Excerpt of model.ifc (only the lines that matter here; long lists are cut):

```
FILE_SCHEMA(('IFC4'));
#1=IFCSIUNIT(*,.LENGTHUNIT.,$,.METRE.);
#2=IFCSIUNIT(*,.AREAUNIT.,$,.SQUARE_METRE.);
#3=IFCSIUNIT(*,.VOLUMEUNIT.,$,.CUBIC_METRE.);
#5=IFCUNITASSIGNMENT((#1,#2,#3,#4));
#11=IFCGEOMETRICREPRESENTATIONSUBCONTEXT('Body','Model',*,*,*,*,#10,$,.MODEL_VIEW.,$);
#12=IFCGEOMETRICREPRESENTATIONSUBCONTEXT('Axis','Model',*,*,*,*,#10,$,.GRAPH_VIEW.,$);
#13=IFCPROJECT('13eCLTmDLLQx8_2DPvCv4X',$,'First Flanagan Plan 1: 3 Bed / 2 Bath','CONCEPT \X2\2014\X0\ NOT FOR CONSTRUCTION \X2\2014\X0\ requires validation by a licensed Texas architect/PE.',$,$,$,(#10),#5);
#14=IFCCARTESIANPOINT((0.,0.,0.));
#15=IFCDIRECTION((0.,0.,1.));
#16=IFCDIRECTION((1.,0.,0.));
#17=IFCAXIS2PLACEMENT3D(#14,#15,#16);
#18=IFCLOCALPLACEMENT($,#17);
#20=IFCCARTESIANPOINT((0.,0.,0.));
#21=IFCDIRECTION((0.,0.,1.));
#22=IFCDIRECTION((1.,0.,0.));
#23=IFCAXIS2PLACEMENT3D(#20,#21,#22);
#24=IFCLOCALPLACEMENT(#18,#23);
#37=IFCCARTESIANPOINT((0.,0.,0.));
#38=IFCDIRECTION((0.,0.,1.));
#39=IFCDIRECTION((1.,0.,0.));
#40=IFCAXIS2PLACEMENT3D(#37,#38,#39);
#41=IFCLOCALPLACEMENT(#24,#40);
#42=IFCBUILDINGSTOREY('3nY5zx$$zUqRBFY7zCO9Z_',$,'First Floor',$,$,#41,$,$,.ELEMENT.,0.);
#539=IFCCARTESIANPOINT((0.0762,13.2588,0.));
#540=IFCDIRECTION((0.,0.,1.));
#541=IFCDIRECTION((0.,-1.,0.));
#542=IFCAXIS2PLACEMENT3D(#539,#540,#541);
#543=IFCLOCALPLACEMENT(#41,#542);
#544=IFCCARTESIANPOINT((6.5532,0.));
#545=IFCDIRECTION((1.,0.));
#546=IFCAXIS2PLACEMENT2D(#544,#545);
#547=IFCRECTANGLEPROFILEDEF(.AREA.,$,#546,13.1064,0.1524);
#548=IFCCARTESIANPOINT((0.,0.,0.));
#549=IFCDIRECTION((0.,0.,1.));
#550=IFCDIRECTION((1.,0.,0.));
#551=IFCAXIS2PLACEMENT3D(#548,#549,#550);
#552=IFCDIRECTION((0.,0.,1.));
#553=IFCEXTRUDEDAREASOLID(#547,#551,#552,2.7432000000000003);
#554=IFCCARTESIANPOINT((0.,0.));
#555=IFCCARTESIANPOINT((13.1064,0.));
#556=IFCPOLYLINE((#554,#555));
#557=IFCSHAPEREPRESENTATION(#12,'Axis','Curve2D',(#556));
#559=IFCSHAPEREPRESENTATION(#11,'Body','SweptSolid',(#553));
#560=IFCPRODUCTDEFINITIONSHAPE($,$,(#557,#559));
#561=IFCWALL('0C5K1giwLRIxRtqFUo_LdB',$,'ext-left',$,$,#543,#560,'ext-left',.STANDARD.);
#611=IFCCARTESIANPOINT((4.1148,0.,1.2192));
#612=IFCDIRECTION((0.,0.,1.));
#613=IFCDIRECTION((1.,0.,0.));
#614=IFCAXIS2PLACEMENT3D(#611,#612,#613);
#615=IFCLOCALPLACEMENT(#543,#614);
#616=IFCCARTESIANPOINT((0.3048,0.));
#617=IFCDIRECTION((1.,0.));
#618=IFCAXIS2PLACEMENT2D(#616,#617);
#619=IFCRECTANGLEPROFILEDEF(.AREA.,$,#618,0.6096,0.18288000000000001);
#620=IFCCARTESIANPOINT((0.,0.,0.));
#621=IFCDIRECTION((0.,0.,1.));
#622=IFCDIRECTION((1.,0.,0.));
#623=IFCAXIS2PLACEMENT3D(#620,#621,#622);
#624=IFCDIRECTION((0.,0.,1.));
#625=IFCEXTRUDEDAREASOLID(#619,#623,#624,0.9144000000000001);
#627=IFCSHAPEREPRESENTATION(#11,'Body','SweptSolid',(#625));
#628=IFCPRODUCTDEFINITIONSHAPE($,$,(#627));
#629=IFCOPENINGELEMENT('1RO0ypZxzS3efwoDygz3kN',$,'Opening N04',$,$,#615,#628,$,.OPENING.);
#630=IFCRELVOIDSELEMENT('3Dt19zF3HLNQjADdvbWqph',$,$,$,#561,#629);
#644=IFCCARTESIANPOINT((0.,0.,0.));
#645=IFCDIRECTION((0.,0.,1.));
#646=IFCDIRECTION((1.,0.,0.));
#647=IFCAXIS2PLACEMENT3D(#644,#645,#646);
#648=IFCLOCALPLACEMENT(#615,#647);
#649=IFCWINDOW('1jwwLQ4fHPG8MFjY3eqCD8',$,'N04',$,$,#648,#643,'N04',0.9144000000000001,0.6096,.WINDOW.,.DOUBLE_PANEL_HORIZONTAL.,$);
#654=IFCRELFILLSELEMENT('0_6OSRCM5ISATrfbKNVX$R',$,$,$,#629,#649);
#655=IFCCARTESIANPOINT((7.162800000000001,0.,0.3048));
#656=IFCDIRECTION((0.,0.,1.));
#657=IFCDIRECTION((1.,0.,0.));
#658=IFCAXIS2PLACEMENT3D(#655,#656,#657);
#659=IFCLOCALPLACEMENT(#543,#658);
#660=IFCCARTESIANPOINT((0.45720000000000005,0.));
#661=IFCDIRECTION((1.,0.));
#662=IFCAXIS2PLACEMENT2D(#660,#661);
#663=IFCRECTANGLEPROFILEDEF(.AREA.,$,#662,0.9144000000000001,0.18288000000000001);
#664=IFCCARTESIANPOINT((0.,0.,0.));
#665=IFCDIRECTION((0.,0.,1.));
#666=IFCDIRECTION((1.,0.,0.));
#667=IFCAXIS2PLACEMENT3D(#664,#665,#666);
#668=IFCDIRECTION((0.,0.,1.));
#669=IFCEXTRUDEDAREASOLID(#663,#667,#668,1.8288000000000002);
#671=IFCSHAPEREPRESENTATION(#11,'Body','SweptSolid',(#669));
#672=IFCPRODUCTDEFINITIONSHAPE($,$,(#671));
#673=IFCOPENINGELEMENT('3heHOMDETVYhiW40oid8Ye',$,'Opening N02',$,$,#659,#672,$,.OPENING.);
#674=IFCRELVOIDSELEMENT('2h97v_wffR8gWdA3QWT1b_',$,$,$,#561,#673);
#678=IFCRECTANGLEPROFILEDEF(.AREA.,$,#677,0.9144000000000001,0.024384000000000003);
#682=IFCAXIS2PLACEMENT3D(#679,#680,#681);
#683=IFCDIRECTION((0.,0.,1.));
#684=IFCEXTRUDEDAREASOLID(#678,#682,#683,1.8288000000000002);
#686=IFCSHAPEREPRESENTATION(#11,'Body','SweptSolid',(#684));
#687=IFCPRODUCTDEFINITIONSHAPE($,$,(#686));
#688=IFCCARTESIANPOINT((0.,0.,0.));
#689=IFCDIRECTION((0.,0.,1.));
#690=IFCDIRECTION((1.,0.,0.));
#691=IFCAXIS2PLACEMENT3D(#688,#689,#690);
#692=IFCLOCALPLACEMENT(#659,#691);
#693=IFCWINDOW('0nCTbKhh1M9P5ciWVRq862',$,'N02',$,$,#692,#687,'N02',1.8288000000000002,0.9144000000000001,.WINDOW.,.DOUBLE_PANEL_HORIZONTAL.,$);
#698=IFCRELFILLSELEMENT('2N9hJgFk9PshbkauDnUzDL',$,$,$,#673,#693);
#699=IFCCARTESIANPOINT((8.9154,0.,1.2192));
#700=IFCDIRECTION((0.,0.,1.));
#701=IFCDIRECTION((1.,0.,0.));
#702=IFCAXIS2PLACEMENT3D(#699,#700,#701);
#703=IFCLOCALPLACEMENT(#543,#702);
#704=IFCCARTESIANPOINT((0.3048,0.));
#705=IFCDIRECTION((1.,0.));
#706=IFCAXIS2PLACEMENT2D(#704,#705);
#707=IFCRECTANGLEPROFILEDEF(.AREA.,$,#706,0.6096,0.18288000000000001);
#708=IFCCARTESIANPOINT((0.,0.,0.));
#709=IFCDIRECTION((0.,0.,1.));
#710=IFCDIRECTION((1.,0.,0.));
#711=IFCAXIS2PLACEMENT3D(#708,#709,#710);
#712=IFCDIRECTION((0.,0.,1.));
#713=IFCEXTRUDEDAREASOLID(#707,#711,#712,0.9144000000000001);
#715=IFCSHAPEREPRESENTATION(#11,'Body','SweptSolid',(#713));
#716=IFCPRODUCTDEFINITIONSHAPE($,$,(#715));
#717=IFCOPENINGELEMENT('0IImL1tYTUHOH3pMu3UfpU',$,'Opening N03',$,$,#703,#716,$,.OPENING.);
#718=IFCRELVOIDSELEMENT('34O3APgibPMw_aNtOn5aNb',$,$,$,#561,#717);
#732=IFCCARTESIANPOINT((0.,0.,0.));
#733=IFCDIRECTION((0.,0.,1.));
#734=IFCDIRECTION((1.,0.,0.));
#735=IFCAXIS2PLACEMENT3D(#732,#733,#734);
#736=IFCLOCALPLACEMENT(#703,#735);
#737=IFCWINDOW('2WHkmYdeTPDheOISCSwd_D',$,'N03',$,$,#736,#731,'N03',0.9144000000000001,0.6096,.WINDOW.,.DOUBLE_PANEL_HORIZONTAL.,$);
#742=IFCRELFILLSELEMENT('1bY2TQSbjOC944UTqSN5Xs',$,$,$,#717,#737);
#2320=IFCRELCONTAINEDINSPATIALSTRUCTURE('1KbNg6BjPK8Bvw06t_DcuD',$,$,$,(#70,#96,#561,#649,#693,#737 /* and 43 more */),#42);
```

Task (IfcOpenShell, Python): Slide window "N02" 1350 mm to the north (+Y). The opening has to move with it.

```python
import ifcopenshell
import ifcopenshell.api.geometry
import ifcopenshell.util.placement

model = ifcopenshell.open("model.ifc")

window = model.by_guid("0nCTbKhh1M9P5ciWVRq862")
opening = window.FillsVoids[0].RelatingOpeningElement
wall = opening.VoidsElements[0].RelatingBuildingElement

wall_matrix = ifcopenshell.util.placement.get_local_placement(wall.ObjectPlacement)
shift = wall_matrix[:3, 0] * -1.35
before = ifcopenshell.util.placement.get_local_placement(window.ObjectPlacement)[:3, 3].copy()

# The window is placed relative to its opening, so it follows when the opening moves.
matrix = ifcopenshell.util.placement.get_local_placement(opening.ObjectPlacement)
matrix[:3, 3] += shift
ifcopenshell.api.geometry.edit_object_placement(
    model, product=opening, matrix=matrix, is_si=False, should_transform_children=True
)

after = ifcopenshell.util.placement.get_local_placement(window.ObjectPlacement)[:3, 3]
print("window moved by", (after - before).round(3) + 0.0)

model.write("model_v2.ifc")
```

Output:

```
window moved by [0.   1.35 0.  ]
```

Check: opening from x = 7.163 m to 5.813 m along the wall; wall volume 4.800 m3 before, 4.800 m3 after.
